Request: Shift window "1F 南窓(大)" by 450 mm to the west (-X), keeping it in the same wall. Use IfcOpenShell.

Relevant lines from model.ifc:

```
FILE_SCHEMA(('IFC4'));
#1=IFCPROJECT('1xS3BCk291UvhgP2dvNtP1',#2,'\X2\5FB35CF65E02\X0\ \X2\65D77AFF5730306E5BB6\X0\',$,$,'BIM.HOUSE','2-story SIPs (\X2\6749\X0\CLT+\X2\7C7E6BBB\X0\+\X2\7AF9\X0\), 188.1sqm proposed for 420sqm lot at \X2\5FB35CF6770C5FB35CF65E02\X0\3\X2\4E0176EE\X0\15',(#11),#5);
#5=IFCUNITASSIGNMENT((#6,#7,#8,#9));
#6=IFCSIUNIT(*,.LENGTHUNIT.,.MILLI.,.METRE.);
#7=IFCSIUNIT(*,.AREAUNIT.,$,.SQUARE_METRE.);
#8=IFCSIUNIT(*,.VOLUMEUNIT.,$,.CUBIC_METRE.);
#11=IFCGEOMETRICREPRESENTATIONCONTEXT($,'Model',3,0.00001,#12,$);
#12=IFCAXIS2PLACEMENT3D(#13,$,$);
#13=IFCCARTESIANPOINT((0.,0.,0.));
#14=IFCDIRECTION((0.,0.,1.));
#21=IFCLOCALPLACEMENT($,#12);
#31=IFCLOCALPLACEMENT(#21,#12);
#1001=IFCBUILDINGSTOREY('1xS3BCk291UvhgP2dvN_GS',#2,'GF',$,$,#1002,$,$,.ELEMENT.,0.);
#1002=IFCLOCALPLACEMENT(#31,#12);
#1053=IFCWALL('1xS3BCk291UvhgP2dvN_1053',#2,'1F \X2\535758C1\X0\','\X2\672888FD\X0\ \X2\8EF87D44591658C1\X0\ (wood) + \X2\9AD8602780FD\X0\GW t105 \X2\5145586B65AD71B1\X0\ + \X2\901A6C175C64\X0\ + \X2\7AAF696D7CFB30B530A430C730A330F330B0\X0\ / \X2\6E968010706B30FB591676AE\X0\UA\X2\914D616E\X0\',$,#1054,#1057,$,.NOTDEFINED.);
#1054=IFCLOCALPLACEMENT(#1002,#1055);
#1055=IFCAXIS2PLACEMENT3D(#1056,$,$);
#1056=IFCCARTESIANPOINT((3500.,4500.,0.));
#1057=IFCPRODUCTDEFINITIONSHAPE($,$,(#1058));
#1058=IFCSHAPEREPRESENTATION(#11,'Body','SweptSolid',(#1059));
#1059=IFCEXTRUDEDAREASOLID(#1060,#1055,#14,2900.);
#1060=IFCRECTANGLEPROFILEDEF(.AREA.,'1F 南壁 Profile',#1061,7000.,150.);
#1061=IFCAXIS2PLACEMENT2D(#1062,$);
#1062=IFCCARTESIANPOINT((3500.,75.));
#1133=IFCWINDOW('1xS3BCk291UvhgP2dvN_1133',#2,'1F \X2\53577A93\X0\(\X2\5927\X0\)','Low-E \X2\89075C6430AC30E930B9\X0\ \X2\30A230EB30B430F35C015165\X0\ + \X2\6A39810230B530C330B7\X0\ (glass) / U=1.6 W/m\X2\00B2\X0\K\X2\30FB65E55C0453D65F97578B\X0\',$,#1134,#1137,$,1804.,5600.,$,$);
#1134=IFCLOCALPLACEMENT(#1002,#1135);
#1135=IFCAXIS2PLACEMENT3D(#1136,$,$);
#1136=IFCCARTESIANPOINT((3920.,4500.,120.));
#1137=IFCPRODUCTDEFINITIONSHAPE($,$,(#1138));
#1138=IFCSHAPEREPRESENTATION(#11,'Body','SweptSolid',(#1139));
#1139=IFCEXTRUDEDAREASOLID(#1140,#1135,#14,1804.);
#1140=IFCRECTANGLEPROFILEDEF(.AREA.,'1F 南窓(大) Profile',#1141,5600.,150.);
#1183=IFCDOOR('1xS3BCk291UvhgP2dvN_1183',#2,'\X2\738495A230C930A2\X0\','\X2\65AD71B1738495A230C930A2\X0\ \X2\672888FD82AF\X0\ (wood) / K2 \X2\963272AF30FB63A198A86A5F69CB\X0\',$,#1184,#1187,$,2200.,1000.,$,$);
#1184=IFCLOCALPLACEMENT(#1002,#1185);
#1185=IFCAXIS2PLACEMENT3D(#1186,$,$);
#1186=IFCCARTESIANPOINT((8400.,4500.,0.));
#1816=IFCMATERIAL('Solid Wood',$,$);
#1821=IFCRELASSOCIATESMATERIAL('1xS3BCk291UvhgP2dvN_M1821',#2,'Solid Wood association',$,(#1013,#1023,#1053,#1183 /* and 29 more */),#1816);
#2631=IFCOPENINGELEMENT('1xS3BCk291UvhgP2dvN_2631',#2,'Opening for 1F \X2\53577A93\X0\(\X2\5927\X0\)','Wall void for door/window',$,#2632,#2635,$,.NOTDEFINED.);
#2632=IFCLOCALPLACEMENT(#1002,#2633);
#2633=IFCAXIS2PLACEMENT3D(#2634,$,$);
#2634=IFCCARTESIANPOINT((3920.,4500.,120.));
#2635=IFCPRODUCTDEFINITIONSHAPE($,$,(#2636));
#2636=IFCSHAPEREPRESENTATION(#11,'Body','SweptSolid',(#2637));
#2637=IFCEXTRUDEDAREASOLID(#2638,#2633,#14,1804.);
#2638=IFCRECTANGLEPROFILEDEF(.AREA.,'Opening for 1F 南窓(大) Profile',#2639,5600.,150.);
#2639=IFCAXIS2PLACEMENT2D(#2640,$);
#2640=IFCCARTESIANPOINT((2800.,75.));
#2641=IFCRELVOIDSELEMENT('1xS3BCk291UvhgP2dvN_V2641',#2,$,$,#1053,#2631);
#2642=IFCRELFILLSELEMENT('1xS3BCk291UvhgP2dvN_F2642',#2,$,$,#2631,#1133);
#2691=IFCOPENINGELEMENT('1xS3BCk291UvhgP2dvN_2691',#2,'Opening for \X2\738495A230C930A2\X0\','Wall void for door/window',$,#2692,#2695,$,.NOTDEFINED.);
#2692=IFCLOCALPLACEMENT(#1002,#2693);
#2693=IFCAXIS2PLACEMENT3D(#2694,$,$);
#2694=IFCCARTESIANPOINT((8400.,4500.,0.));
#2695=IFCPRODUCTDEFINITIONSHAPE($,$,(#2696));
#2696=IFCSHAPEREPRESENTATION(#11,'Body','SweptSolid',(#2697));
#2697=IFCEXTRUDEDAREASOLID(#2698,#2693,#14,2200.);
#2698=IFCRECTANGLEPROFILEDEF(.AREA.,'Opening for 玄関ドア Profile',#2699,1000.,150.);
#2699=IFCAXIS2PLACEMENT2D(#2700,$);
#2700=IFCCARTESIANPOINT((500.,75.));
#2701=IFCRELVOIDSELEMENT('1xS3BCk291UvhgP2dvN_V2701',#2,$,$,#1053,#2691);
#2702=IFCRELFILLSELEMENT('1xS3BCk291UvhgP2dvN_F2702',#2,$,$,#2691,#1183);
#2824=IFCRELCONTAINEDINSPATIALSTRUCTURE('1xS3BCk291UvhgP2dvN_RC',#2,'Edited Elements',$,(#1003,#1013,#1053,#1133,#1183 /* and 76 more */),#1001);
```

```python
import ifcopenshell
import ifcopenshell.api.geometry
import ifcopenshell.util.placement

model = ifcopenshell.open("model.ifc")

window = model.by_guid("1xS3BCk291UvhgP2dvN_1133")
opening = window.FillsVoids[0].RelatingOpeningElement
wall = opening.VoidsElements[0].RelatingBuildingElement

wall_matrix = ifcopenshell.util.placement.get_local_placement(wall.ObjectPlacement)
shift = wall_matrix[:3, 0] * -450.0
before = ifcopenshell.util.placement.get_local_placement(window.ObjectPlacement)[:3, 3].copy()

# The window is not placed relative to its opening, so move both.
for product in (opening, window):
    matrix = ifcopenshell.util.placement.get_local_placement(product.ObjectPlacement)
    matrix[:3, 3] += shift
    ifcopenshell.api.geometry.edit_object_placement(model, product=product, matrix=matrix, is_si=False)

after = ifcopenshell.util.placement.get_local_placement(window.ObjectPlacement)[:3, 3]
print("window moved by", (after - before).round(3) + 0.0)

model.write("model_edited.ifc")
```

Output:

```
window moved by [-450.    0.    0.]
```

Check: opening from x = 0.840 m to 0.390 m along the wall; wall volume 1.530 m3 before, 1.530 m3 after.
